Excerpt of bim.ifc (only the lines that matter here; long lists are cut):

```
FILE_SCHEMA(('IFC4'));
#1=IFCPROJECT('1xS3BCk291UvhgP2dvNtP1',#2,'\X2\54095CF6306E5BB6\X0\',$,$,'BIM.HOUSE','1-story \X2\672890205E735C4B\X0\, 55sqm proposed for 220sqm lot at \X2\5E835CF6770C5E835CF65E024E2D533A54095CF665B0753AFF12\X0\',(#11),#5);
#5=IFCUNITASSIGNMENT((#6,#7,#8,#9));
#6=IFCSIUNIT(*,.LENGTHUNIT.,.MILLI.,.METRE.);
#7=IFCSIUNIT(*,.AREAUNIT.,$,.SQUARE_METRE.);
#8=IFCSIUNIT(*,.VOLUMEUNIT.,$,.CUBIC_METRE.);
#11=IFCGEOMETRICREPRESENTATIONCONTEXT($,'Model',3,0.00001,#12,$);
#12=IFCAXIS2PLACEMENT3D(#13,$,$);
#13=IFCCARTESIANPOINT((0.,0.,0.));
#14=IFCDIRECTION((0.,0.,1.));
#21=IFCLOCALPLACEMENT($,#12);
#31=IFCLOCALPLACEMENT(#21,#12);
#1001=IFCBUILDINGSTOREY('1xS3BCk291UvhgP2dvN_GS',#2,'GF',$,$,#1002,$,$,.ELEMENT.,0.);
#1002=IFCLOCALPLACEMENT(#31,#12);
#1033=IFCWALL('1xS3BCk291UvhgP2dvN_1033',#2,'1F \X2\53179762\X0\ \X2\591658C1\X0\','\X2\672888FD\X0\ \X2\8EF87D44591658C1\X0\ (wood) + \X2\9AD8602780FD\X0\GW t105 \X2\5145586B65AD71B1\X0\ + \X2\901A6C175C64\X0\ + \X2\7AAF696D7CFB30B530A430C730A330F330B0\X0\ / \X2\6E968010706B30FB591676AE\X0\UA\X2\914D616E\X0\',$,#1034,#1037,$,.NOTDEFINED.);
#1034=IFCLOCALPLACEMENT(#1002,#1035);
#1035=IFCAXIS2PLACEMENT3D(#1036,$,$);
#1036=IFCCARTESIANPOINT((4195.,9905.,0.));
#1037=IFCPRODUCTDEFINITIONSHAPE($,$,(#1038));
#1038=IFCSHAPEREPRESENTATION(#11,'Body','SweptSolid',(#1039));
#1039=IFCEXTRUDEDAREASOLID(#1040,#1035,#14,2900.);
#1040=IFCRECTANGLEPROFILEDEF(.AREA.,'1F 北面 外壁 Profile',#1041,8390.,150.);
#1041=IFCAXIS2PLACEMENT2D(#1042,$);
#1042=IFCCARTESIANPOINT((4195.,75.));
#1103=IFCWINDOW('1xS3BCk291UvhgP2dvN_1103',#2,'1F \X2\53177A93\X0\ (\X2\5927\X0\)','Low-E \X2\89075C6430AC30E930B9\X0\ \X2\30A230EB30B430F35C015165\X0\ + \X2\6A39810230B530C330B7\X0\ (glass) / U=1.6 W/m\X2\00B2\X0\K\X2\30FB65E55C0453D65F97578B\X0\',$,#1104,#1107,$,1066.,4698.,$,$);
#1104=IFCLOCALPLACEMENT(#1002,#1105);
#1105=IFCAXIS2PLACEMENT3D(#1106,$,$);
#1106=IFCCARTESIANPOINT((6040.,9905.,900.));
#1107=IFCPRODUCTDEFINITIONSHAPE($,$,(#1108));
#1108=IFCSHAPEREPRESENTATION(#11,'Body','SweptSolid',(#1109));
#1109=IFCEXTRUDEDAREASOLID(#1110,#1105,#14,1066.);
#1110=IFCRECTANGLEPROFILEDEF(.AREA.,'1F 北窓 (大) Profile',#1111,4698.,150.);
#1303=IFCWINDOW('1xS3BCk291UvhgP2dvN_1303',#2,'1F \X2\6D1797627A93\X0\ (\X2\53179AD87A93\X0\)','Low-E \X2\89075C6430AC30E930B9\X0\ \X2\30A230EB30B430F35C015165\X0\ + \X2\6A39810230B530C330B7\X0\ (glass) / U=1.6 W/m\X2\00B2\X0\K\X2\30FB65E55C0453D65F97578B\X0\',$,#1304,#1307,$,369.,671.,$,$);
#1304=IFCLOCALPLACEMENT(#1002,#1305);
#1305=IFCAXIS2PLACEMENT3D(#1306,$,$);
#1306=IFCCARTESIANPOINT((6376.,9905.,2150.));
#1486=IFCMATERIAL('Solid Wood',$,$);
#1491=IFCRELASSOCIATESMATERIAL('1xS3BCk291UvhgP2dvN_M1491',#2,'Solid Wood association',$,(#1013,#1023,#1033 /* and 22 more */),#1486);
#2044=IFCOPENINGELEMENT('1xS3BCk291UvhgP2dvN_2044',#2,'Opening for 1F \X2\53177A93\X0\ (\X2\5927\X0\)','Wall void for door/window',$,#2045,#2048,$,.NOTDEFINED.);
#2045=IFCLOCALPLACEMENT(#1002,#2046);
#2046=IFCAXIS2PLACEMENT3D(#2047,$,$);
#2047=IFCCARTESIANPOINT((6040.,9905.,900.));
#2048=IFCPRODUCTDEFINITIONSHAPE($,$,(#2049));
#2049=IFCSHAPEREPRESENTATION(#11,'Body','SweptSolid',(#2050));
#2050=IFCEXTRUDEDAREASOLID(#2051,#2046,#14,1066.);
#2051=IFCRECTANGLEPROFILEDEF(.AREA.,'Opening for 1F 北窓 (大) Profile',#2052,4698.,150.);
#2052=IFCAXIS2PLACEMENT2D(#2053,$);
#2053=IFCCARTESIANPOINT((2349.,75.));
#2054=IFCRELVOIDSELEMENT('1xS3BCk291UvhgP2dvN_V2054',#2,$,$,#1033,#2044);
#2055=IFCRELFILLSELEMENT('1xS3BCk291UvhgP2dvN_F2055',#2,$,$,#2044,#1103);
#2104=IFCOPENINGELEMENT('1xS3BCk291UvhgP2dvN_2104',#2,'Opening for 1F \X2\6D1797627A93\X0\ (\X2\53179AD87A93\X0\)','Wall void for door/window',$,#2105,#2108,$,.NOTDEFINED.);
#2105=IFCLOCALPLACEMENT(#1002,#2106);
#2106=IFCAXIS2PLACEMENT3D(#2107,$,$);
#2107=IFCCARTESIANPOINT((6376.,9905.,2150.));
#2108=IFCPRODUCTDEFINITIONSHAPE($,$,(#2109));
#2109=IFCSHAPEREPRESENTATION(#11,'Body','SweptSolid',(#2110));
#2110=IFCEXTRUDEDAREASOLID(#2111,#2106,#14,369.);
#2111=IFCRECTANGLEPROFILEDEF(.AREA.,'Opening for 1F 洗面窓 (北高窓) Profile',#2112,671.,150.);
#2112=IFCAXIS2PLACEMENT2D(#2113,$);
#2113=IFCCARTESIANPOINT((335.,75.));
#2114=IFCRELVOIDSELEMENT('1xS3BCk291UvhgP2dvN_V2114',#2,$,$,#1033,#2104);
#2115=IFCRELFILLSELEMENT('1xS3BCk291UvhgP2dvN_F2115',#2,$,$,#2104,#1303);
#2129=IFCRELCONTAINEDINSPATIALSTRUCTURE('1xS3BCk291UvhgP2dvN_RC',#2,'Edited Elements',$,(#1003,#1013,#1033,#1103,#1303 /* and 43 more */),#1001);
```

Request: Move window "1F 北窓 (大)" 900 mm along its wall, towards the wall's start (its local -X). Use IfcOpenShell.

```python
import ifcopenshell
import ifcopenshell.api.geometry
import ifcopenshell.util.placement

model = ifcopenshell.open("bim.ifc")

window = model.by_guid("1xS3BCk291UvhgP2dvN_1103")
opening = window.FillsVoids[0].RelatingOpeningElement
wall = opening.VoidsElements[0].RelatingBuildingElement

wall_matrix = ifcopenshell.util.placement.get_local_placement(wall.ObjectPlacement)
shift = wall_matrix[:3, 0] * -900.0
before = ifcopenshell.util.placement.get_local_placement(window.ObjectPlacement)[:3, 3].copy()

# The window is not placed relative to its opening, so move both.
for product in (opening, window):
    matrix = ifcopenshell.util.placement.get_local_placement(product.ObjectPlacement)
    matrix[:3, 3] += shift
    ifcopenshell.api.geometry.edit_object_placement(model, product=product, matrix=matrix, is_si=False)

after = ifcopenshell.util.placement.get_local_placement(window.ObjectPlacement)[:3, 3]
print("window moved by", (after - before).round(3) + 0.0)

model.write("bim_rev.ifc")
```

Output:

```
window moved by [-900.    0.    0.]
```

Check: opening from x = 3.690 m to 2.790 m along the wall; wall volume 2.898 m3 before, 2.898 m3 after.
